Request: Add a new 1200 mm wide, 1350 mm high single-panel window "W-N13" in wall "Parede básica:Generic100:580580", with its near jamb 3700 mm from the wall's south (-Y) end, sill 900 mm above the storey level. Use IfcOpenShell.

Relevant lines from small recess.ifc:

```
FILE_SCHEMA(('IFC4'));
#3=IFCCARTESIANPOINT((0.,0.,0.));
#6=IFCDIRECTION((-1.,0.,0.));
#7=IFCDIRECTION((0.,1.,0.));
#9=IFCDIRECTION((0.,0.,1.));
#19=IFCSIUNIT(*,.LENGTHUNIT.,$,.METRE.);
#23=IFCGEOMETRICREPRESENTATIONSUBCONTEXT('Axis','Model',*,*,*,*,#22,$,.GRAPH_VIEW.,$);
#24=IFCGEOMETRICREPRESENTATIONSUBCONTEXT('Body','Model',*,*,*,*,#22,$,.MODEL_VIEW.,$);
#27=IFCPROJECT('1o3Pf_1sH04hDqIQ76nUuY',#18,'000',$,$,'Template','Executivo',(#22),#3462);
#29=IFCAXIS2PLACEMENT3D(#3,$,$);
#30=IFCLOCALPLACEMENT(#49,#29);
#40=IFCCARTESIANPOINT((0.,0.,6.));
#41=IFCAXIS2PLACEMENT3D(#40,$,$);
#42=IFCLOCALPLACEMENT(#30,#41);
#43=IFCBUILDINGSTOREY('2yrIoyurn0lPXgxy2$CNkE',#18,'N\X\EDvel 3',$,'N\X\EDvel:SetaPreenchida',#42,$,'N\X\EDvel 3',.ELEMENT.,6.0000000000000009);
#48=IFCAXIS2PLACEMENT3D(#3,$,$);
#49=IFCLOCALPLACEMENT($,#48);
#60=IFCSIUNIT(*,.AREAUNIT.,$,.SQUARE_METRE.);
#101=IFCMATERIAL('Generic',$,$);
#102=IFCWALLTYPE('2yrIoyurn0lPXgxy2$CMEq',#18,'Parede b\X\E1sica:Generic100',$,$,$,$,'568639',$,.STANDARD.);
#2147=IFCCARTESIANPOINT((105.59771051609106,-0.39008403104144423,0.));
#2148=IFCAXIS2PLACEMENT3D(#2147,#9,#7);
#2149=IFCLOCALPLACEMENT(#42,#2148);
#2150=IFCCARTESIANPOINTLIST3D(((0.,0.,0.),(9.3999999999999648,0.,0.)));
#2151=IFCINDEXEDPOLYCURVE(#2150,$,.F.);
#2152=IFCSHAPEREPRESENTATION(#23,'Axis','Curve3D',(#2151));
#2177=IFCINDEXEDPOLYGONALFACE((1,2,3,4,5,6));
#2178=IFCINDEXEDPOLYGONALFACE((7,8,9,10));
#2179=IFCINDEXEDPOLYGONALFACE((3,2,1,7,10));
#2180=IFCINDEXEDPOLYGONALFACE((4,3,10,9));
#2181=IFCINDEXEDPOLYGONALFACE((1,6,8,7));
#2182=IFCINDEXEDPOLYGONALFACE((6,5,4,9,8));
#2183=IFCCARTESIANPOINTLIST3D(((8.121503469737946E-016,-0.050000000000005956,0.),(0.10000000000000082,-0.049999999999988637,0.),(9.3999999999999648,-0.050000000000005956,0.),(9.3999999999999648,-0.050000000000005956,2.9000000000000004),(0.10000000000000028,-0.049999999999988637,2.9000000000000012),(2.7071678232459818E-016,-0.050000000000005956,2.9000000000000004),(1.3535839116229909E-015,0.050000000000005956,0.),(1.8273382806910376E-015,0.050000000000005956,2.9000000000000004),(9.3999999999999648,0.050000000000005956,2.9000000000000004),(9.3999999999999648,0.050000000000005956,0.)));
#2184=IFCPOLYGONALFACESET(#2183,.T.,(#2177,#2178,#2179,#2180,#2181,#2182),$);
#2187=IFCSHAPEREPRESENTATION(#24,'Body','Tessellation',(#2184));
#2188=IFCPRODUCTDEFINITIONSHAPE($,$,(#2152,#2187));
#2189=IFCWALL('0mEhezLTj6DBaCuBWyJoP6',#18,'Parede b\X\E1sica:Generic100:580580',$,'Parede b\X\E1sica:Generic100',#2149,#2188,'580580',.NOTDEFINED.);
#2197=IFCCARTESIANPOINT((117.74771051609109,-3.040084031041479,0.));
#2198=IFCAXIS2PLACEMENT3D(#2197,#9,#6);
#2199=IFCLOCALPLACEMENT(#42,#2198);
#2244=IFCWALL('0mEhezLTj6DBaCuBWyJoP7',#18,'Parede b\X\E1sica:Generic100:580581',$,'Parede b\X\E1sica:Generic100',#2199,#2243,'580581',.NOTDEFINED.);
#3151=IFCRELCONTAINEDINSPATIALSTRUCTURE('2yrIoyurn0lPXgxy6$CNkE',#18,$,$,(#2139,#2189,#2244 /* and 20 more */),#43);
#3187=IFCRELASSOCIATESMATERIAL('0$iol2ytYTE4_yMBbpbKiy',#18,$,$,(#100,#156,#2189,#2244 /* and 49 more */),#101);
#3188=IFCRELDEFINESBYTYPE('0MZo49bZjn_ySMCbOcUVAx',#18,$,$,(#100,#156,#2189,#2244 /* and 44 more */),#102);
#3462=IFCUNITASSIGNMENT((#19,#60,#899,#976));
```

```python
import numpy as np
import ifcopenshell
import ifcopenshell.api.feature
import ifcopenshell.api.geometry
import ifcopenshell.api.root
import ifcopenshell.api.spatial
import ifcopenshell.geom
import ifcopenshell.util.element
import ifcopenshell.util.placement
import ifcopenshell.util.representation
import ifcopenshell.util.shape
import ifcopenshell.util.unit

model = ifcopenshell.open("small recess.ifc")
unit_scale = ifcopenshell.util.unit.calculate_unit_scale(model)
settings = ifcopenshell.geom.settings()


def volume(element):
    """Net volume in cubic metres, openings subtracted."""
    shape = ifcopenshell.geom.create_shape(settings, element)
    return ifcopenshell.util.shape.get_volume(shape.geometry)


wall = model.by_guid("0mEhezLTj6DBaCuBWyJoP6")
storey = ifcopenshell.util.element.get_container(wall, ifc_class="IfcBuildingStorey")
context = ifcopenshell.util.representation.get_context(model, "Model", "Body", "MODEL_VIEW")
before = volume(wall)

width, height, from_end, sill = 1.2, 1.35, 3.7, 0.9  # metres

# The wall runs along its own X axis, and the end named is its -X end.
wall_shape = ifcopenshell.geom.create_shape(settings, wall)
x, y, z = ifcopenshell.util.shape.get_vertices(wall_shape.geometry).T
start = x.min() + from_end
face, thickness = float(y.min()), float(y.max() - y.min())
wall_matrix = ifcopenshell.util.placement.get_local_placement(wall.ObjectPlacement)
level = ifcopenshell.util.placement.get_local_placement(storey.ObjectPlacement)[2, 3]


def in_wall(x, y):
    """Placement at x, y metres in the wall's axes, at sill height."""
    matrix = wall_matrix.copy()
    matrix[:, 3] = wall_matrix @ np.array([x / unit_scale, y / unit_scale, 0.0, 1.0])
    matrix[2, 3] = level + sill / unit_scale
    return matrix


# Opening: a box that overshoots both wall faces by 50 mm.
opening = ifcopenshell.api.root.create_entity(model, ifc_class="IfcOpeningElement", predefined_type="OPENING")
box = ifcopenshell.api.geometry.add_wall_representation(
    model, context=context, length=width, height=height, thickness=thickness + 0.1
)
ifcopenshell.api.geometry.assign_representation(model, product=opening, representation=box)
ifcopenshell.api.geometry.edit_object_placement(model, product=opening, matrix=in_wall(start, face - 0.05), is_si=False)
ifcopenshell.api.feature.add_feature(model, feature=opening, element=wall)

window = ifcopenshell.api.root.create_entity(model, ifc_class="IfcWindow", name="W-N13", predefined_type="WINDOW")
window.OverallWidth, window.OverallHeight = width / unit_scale, height / unit_scale
window.PartitioningType = "SINGLE_PANEL"
body = ifcopenshell.api.geometry.add_window_representation(
    model,
    context=context,
    overall_width=window.OverallWidth,
    overall_height=window.OverallHeight,
    partition_type="SINGLE_PANEL",
)
ifcopenshell.api.geometry.assign_representation(model, product=window, representation=body)
ifcopenshell.api.spatial.assign_container(model, products=[window], relating_structure=storey)
ifcopenshell.api.feature.add_filling(model, opening=opening, element=window)

# Centre the window in the wall's thickness.
ifcopenshell.api.geometry.edit_object_placement(model, product=window, matrix=in_wall(start, face), is_si=False)
window_shape = ifcopenshell.geom.create_shape(settings, window)
depth = ifcopenshell.util.shape.get_vertices(window_shape.geometry)[:, 1]
offset = face + thickness / 2 - (depth.min() + depth.max()) / 2
ifcopenshell.api.geometry.edit_object_placement(model, product=window, matrix=in_wall(start, offset), is_si=False)

after = volume(wall)

print(f"wall volume {before:.3f} -> {after:.3f} m3")

model.write("small recess-out.ifc")
```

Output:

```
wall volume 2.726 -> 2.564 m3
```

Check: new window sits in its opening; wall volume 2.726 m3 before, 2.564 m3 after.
